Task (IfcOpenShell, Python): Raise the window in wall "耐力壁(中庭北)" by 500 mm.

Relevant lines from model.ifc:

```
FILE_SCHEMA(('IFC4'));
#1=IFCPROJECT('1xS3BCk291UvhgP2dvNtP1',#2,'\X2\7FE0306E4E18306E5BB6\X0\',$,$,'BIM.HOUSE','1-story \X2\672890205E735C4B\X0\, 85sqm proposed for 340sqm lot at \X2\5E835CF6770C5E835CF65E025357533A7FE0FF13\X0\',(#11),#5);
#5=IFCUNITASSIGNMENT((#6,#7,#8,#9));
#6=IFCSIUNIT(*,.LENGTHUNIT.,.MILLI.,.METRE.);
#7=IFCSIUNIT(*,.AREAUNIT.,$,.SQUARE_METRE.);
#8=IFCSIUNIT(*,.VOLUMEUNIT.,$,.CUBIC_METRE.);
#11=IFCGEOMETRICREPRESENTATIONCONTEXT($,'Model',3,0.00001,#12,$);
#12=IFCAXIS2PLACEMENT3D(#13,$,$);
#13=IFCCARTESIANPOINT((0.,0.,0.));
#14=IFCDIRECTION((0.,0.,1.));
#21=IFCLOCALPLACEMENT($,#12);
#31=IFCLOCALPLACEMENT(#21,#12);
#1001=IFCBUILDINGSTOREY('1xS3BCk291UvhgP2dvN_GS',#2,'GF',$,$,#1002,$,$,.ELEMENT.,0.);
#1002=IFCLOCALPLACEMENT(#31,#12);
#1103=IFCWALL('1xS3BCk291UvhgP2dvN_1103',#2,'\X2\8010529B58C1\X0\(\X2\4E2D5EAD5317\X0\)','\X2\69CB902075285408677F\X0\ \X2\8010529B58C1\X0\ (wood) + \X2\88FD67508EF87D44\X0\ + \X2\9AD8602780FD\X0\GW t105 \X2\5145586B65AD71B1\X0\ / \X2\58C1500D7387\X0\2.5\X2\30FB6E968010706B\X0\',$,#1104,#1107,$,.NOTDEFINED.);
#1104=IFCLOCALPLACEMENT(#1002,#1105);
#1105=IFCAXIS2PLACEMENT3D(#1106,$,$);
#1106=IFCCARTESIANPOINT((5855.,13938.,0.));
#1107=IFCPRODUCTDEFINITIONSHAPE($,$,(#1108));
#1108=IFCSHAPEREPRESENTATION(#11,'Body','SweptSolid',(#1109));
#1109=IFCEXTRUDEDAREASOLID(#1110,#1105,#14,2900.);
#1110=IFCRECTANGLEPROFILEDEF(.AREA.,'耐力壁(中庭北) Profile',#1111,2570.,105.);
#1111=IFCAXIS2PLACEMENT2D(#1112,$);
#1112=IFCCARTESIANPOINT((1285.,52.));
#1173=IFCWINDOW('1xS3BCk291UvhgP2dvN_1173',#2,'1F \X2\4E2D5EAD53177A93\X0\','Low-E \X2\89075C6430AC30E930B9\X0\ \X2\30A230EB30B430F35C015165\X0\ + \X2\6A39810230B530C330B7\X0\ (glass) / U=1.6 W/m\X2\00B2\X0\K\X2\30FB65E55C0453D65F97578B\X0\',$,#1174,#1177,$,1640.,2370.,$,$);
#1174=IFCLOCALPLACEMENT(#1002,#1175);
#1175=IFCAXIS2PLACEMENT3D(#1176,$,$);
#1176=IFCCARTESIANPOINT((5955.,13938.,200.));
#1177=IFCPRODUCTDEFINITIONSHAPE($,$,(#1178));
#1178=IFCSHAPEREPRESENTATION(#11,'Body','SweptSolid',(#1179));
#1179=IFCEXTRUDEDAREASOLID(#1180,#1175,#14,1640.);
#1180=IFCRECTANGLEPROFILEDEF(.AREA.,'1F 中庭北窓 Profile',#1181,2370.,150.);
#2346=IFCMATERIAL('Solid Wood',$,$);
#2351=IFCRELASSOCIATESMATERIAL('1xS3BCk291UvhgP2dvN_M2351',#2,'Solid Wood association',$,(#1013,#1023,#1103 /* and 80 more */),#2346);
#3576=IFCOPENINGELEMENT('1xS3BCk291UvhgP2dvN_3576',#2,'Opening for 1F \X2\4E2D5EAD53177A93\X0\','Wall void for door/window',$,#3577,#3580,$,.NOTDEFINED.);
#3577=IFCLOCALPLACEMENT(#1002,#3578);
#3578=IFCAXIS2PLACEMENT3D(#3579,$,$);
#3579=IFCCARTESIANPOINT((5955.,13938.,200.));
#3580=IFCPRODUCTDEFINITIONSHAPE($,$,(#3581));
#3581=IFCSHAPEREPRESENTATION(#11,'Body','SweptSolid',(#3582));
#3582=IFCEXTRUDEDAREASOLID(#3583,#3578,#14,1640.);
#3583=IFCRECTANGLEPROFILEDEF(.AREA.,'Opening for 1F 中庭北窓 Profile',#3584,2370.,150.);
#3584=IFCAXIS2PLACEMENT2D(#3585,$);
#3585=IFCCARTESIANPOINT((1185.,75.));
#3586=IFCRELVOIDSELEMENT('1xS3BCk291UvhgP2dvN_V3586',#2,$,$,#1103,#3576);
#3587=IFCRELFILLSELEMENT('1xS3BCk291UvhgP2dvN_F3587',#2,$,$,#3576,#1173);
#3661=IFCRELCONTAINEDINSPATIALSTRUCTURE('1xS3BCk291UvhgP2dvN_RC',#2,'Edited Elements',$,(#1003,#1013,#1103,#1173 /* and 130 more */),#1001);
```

```python
import numpy as np
import ifcopenshell
import ifcopenshell.api.geometry
import ifcopenshell.util.placement
import ifcopenshell.util.unit

model = ifcopenshell.open("model.ifc")
unit_scale = ifcopenshell.util.unit.calculate_unit_scale(model)

window = model.by_guid("1xS3BCk291UvhgP2dvN_1173")
opening = window.FillsVoids[0].RelatingOpeningElement
dz = 0.5 / unit_scale

shift = np.array([0.0, 0.0, dz])
# The window is not placed relative to its opening, so move both.
for product in (opening, window):
    matrix = ifcopenshell.util.placement.get_local_placement(product.ObjectPlacement)
    matrix[:3, 3] += shift
    ifcopenshell.api.geometry.edit_object_placement(model, product=product, matrix=matrix, is_si=False)

print(f"moved by {dz * unit_scale:+.3f} m")

model.write("model_rev.ifc")
```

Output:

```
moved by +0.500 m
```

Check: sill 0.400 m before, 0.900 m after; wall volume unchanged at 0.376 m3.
